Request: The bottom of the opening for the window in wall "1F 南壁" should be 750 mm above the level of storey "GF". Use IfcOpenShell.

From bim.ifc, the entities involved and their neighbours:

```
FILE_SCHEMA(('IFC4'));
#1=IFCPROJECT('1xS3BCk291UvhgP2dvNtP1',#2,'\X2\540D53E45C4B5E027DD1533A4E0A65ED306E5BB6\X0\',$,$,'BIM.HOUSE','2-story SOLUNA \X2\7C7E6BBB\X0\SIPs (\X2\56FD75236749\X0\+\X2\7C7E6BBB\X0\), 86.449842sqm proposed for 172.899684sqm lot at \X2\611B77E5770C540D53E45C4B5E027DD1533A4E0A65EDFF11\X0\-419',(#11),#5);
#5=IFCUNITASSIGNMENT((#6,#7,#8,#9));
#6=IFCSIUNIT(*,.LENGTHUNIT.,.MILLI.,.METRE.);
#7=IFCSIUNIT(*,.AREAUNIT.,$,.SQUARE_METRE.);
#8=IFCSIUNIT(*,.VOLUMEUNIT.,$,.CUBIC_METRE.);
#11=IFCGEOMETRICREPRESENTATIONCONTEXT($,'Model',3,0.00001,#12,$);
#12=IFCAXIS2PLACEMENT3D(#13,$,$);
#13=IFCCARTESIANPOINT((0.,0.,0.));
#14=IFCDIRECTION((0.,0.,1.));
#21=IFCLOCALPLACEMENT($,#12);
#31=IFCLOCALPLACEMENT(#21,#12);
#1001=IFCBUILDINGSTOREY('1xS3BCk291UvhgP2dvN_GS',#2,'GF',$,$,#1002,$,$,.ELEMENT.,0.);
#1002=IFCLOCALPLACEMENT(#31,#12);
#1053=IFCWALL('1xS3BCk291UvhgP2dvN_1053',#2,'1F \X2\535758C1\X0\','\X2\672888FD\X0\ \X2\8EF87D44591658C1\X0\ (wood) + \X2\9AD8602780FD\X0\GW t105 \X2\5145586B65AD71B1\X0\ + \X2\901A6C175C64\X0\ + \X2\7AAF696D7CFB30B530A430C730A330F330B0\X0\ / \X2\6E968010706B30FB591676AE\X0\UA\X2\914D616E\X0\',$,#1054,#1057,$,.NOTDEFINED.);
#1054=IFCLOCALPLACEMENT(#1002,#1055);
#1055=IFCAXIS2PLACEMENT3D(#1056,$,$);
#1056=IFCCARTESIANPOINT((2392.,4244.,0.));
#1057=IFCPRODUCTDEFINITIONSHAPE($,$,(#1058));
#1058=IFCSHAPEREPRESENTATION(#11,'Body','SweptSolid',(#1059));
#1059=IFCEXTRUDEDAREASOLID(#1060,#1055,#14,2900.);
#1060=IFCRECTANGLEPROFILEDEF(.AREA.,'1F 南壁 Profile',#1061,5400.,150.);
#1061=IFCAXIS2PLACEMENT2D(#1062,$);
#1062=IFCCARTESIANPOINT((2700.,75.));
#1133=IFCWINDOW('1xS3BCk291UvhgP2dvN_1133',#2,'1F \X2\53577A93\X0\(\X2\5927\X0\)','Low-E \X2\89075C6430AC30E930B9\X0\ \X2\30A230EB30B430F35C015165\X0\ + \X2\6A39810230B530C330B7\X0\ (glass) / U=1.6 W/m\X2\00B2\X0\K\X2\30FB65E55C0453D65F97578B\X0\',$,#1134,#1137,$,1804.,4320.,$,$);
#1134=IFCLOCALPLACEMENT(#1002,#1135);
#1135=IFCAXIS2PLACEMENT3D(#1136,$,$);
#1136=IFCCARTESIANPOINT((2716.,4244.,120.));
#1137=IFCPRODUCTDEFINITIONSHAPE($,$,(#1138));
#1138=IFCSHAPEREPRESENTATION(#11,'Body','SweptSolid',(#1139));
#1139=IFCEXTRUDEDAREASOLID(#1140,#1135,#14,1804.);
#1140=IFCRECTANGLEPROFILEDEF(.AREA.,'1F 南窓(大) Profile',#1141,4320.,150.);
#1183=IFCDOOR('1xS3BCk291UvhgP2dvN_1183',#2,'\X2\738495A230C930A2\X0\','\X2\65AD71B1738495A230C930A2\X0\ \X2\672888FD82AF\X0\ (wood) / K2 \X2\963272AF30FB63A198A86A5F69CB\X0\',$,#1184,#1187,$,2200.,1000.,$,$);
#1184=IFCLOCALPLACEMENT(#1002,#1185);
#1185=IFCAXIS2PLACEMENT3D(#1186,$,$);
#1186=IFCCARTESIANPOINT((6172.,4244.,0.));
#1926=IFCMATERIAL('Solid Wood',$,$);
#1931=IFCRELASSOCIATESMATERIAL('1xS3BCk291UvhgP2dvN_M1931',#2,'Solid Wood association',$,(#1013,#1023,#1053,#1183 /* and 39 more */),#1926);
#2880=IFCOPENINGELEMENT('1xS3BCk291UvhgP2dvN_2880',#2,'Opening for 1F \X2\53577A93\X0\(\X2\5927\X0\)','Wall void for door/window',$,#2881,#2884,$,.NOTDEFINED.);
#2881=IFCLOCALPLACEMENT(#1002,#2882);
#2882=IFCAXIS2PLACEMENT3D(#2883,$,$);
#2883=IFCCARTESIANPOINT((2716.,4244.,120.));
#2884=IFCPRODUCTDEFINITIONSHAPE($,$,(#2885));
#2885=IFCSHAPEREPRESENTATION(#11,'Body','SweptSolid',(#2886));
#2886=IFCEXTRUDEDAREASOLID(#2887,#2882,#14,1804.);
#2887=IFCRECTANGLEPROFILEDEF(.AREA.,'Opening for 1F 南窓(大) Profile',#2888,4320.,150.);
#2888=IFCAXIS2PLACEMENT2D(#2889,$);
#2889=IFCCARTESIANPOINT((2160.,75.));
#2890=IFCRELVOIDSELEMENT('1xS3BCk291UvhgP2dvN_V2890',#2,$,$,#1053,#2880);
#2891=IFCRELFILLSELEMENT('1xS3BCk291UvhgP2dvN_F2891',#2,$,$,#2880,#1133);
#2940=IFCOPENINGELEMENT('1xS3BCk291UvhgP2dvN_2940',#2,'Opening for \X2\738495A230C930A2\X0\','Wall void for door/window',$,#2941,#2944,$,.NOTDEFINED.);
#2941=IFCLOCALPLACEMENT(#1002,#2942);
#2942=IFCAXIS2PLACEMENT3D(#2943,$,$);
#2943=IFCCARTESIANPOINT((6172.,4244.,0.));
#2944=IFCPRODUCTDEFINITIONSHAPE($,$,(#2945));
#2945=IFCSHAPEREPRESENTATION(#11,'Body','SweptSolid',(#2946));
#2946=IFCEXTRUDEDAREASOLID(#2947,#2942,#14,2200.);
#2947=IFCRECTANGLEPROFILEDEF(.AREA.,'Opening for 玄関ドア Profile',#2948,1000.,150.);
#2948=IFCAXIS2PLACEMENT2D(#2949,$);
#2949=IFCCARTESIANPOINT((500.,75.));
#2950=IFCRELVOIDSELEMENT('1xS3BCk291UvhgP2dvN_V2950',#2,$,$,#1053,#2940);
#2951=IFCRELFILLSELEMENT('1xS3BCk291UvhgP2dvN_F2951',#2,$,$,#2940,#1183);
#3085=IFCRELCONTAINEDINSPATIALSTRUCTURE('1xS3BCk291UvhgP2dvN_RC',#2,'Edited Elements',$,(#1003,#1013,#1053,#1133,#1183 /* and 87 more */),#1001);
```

```python
import numpy as np
import ifcopenshell
import ifcopenshell.api.geometry
import ifcopenshell.geom
import ifcopenshell.util.element
import ifcopenshell.util.placement
import ifcopenshell.util.shape
import ifcopenshell.util.unit

model = ifcopenshell.open("bim.ifc")
unit_scale = ifcopenshell.util.unit.calculate_unit_scale(model)

window = model.by_id(1133)
opening = window.FillsVoids[0].RelatingOpeningElement
storey = ifcopenshell.util.element.get_container(window, ifc_class="IfcBuildingStorey")
level = ifcopenshell.util.placement.get_local_placement(storey.ObjectPlacement)[2, 3]

# The opening's origin need not be at the sill, so measure its lowest point.
shape = ifcopenshell.geom.create_shape(ifcopenshell.geom.settings(), opening)
bottom = ifcopenshell.util.shape.get_shape_bottom_elevation(shape, shape.geometry) / unit_scale
dz = level + 0.75 / unit_scale - bottom

shift = np.array([0.0, 0.0, dz])
# The window is not placed relative to its opening, so move both.
for product in (opening, window):
    matrix = ifcopenshell.util.placement.get_local_placement(product.ObjectPlacement)
    matrix[:3, 3] += shift
    ifcopenshell.api.geometry.edit_object_placement(model, product=product, matrix=matrix, is_si=False)

print(f"moved by {dz * unit_scale:+.3f} m")

model.write("bim-out.ifc")
```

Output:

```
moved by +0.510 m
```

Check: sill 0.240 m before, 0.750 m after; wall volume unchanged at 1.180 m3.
